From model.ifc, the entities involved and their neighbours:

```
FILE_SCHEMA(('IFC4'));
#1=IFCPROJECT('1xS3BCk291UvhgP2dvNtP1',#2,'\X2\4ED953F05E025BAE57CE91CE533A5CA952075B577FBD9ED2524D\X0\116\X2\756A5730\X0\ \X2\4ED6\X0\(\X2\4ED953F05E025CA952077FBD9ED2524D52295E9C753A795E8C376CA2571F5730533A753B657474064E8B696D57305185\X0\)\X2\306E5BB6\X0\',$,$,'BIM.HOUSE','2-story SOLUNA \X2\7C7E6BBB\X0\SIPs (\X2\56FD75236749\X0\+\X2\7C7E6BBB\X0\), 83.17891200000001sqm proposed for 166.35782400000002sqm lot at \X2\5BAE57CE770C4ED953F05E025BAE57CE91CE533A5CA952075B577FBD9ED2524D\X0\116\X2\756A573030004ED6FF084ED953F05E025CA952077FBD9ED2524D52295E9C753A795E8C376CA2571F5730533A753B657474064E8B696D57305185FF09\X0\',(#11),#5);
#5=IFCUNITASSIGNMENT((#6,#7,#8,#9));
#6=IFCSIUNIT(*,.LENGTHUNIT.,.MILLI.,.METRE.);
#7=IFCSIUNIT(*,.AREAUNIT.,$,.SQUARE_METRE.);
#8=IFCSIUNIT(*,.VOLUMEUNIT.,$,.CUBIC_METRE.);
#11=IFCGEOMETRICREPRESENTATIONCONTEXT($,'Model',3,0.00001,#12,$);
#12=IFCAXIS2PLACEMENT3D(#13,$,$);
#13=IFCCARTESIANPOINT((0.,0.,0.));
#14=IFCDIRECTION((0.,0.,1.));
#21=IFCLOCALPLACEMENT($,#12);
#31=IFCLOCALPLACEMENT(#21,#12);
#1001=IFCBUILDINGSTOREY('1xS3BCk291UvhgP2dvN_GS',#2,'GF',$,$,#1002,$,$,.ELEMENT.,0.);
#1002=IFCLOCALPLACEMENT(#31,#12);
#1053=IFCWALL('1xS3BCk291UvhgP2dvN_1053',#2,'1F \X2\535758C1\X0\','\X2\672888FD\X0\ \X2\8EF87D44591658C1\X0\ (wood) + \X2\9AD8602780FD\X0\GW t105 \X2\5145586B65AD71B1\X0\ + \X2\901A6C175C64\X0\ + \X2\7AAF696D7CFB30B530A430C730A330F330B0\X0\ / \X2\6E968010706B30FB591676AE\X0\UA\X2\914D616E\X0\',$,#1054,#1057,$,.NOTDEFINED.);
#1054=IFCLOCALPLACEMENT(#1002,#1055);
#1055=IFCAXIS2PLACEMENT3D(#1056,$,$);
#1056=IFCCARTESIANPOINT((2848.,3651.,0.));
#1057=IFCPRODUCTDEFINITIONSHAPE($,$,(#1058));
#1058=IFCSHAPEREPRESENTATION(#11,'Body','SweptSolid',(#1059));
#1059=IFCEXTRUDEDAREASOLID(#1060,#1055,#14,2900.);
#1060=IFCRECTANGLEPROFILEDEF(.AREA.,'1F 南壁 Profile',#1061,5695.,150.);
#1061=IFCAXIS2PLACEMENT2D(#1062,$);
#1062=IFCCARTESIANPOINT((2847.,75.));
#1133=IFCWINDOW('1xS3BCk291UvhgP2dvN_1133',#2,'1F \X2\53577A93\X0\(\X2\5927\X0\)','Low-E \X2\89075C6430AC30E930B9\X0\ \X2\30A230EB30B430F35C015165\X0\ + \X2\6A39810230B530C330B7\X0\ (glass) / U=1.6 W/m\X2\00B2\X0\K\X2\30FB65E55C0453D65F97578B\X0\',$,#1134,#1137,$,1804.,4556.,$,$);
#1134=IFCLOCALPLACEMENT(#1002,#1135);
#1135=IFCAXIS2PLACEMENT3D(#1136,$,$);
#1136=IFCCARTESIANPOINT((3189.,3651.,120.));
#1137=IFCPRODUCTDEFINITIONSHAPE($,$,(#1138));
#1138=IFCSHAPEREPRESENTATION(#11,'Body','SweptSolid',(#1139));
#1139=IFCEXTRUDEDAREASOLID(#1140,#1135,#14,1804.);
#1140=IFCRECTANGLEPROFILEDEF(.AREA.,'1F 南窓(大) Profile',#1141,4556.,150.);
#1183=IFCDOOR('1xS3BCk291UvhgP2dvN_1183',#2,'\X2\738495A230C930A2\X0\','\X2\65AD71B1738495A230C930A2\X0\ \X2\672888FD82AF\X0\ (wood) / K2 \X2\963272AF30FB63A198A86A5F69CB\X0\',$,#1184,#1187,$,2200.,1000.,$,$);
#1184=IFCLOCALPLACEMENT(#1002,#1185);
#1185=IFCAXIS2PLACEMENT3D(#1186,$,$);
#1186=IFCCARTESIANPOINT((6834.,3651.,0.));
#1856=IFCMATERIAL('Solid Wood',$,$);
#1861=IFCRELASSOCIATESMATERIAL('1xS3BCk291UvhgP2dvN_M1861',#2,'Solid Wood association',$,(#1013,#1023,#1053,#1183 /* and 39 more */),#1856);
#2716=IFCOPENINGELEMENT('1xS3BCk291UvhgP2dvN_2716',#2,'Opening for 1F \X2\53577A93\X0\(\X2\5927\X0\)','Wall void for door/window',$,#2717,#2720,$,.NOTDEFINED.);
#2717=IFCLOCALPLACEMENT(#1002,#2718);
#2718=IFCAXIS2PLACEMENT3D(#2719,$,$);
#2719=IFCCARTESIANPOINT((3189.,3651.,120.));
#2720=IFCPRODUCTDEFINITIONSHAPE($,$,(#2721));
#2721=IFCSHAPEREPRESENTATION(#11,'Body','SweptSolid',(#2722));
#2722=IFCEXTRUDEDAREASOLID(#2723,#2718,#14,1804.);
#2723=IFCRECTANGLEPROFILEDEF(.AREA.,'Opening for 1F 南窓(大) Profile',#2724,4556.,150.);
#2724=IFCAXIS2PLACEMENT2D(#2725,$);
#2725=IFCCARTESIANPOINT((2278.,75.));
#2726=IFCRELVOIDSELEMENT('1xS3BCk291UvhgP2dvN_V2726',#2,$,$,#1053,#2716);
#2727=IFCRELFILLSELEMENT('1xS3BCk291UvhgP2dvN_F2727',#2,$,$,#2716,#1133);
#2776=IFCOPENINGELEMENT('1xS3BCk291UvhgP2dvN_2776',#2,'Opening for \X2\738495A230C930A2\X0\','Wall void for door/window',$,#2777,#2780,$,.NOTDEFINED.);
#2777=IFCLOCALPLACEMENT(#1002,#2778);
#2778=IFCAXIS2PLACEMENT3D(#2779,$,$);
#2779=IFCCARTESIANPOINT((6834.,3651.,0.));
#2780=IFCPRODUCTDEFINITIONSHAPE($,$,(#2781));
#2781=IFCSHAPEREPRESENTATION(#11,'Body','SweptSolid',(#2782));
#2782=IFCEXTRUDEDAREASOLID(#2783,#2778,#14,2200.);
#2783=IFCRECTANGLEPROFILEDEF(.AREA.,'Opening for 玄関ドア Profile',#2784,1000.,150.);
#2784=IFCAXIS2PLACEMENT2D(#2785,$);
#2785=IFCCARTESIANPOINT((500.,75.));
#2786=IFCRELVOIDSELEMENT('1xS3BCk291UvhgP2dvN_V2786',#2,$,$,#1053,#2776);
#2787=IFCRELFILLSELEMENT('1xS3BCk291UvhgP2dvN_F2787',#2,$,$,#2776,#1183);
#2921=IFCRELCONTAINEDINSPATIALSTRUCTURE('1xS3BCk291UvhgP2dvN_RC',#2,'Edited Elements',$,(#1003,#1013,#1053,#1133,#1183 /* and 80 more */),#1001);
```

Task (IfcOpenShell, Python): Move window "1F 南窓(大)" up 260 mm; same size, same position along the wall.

```python
import numpy as np
import ifcopenshell
import ifcopenshell.api.geometry
import ifcopenshell.util.placement
import ifcopenshell.util.unit

model = ifcopenshell.open("model.ifc")
unit_scale = ifcopenshell.util.unit.calculate_unit_scale(model)

window = model.by_guid("1xS3BCk291UvhgP2dvN_1133")
opening = window.FillsVoids[0].RelatingOpeningElement
dz = 260.0

shift = np.array([0.0, 0.0, dz])
# The window is not placed relative to its opening, so move both.
for product in (opening, window):
    matrix = ifcopenshell.util.placement.get_local_placement(product.ObjectPlacement)
    matrix[:3, 3] += shift
    ifcopenshell.api.geometry.edit_object_placement(model, product=product, matrix=matrix, is_si=False)

print(f"moved by {dz * unit_scale:+.3f} m")

model.write("model_rev.ifc")
```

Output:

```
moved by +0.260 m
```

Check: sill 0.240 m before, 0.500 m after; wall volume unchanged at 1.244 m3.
